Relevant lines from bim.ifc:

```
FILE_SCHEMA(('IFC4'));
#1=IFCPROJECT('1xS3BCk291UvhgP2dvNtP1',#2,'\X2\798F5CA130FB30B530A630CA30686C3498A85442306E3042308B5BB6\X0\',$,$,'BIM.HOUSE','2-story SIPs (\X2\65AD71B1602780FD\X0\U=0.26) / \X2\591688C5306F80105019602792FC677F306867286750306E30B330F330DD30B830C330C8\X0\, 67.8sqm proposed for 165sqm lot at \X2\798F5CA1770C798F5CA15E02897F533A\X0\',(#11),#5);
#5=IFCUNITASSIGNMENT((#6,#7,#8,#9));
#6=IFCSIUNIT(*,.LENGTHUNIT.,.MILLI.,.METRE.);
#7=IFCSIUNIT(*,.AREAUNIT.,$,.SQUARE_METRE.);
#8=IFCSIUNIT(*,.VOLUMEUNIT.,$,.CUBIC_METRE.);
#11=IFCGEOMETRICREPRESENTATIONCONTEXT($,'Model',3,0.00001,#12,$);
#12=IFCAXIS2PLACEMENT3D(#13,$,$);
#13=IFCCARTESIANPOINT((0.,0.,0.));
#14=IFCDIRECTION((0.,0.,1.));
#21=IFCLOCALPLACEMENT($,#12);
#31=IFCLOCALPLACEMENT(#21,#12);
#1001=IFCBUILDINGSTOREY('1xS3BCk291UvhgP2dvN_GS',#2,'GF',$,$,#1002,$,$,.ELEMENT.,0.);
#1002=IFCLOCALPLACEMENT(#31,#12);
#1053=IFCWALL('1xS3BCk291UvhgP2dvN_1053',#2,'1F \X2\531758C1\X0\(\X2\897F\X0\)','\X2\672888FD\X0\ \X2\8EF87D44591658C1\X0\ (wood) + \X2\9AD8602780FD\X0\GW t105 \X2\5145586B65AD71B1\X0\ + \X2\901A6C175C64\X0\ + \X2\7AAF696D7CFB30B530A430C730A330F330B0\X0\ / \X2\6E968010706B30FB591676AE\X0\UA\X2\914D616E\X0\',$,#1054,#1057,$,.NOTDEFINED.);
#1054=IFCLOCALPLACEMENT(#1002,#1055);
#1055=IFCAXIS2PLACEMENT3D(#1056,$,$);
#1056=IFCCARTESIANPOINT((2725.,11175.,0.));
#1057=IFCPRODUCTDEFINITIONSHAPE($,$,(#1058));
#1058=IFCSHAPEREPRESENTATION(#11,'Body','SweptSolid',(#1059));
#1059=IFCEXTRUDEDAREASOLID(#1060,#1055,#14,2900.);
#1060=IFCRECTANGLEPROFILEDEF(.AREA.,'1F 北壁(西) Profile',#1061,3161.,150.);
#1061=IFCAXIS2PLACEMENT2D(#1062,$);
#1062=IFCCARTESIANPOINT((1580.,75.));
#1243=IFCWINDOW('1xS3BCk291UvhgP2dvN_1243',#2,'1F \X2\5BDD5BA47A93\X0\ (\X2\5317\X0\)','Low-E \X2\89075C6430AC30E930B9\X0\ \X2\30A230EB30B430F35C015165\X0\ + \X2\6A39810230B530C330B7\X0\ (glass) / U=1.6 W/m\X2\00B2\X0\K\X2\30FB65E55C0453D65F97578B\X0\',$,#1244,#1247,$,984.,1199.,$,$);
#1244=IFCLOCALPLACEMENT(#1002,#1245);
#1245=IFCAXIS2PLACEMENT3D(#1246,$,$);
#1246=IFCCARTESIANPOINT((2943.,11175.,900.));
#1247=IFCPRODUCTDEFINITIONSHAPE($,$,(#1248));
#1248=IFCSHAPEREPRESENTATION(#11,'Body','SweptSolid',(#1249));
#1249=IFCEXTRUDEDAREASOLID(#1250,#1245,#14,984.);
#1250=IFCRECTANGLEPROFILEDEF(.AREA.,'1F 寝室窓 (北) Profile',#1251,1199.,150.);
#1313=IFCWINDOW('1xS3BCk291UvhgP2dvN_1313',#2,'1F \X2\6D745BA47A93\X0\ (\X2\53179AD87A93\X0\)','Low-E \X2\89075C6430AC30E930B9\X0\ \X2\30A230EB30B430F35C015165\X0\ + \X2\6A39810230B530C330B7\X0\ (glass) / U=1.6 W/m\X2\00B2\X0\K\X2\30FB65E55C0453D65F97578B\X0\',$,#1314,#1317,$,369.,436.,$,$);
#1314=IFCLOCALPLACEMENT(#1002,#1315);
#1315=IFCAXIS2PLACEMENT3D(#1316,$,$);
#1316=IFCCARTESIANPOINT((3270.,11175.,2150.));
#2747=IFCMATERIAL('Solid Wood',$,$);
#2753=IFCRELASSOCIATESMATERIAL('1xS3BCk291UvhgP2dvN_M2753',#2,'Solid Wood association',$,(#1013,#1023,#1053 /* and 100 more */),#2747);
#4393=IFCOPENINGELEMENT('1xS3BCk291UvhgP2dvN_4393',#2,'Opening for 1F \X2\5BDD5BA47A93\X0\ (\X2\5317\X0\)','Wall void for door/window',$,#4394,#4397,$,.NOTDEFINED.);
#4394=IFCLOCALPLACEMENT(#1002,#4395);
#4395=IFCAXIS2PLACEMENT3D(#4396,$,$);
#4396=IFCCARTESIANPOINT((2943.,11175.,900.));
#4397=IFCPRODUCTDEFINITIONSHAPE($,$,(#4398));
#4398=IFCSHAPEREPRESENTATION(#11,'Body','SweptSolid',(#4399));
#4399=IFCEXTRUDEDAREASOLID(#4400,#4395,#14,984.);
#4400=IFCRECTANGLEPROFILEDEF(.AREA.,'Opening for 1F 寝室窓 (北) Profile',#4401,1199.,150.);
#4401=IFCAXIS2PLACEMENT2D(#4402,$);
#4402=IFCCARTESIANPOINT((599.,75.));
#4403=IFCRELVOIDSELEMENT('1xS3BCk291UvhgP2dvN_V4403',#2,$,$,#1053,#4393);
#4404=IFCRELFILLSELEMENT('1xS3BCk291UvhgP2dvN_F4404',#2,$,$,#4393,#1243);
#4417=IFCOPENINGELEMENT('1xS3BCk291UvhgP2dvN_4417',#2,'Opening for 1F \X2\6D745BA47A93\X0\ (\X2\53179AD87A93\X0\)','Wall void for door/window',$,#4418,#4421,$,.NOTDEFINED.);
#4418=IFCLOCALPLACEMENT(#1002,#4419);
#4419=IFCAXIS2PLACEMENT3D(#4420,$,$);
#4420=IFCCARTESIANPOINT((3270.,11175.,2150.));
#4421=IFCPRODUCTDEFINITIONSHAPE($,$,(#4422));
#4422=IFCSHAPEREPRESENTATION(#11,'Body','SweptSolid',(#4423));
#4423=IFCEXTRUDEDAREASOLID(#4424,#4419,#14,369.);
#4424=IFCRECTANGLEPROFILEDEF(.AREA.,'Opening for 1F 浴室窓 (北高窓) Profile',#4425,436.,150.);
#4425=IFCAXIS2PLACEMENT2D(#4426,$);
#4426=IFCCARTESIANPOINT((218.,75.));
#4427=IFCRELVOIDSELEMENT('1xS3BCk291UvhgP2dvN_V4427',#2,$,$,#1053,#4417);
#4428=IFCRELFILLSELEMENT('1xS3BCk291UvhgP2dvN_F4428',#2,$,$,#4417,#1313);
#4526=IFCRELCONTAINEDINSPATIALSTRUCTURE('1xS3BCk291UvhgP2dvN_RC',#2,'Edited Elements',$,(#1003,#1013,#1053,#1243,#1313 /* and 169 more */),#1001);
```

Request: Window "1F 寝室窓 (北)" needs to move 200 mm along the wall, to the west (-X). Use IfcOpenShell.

```python
import ifcopenshell
import ifcopenshell.api.geometry
import ifcopenshell.util.placement
import ifcopenshell.util.unit

model = ifcopenshell.open("bim.ifc")
unit_scale = ifcopenshell.util.unit.calculate_unit_scale(model)

window = model.by_id(1243)
opening = window.FillsVoids[0].RelatingOpeningElement
wall = opening.VoidsElements[0].RelatingBuildingElement

wall_matrix = ifcopenshell.util.placement.get_local_placement(wall.ObjectPlacement)
shift = wall_matrix[:3, 0] * -0.2 / unit_scale
before = ifcopenshell.util.placement.get_local_placement(window.ObjectPlacement)[:3, 3].copy()

# The window is not placed relative to its opening, so move both.
for product in (opening, window):
    matrix = ifcopenshell.util.placement.get_local_placement(product.ObjectPlacement)
    matrix[:3, 3] += shift
    ifcopenshell.api.geometry.edit_object_placement(model, product=product, matrix=matrix, is_si=False)

after = ifcopenshell.util.placement.get_local_placement(window.ObjectPlacement)[:3, 3]
print("window moved by", (after - before).round(3) + 0.0)

model.write("bim_edited.ifc")
```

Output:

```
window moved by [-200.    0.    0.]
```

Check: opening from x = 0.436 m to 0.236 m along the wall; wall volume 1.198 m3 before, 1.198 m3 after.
